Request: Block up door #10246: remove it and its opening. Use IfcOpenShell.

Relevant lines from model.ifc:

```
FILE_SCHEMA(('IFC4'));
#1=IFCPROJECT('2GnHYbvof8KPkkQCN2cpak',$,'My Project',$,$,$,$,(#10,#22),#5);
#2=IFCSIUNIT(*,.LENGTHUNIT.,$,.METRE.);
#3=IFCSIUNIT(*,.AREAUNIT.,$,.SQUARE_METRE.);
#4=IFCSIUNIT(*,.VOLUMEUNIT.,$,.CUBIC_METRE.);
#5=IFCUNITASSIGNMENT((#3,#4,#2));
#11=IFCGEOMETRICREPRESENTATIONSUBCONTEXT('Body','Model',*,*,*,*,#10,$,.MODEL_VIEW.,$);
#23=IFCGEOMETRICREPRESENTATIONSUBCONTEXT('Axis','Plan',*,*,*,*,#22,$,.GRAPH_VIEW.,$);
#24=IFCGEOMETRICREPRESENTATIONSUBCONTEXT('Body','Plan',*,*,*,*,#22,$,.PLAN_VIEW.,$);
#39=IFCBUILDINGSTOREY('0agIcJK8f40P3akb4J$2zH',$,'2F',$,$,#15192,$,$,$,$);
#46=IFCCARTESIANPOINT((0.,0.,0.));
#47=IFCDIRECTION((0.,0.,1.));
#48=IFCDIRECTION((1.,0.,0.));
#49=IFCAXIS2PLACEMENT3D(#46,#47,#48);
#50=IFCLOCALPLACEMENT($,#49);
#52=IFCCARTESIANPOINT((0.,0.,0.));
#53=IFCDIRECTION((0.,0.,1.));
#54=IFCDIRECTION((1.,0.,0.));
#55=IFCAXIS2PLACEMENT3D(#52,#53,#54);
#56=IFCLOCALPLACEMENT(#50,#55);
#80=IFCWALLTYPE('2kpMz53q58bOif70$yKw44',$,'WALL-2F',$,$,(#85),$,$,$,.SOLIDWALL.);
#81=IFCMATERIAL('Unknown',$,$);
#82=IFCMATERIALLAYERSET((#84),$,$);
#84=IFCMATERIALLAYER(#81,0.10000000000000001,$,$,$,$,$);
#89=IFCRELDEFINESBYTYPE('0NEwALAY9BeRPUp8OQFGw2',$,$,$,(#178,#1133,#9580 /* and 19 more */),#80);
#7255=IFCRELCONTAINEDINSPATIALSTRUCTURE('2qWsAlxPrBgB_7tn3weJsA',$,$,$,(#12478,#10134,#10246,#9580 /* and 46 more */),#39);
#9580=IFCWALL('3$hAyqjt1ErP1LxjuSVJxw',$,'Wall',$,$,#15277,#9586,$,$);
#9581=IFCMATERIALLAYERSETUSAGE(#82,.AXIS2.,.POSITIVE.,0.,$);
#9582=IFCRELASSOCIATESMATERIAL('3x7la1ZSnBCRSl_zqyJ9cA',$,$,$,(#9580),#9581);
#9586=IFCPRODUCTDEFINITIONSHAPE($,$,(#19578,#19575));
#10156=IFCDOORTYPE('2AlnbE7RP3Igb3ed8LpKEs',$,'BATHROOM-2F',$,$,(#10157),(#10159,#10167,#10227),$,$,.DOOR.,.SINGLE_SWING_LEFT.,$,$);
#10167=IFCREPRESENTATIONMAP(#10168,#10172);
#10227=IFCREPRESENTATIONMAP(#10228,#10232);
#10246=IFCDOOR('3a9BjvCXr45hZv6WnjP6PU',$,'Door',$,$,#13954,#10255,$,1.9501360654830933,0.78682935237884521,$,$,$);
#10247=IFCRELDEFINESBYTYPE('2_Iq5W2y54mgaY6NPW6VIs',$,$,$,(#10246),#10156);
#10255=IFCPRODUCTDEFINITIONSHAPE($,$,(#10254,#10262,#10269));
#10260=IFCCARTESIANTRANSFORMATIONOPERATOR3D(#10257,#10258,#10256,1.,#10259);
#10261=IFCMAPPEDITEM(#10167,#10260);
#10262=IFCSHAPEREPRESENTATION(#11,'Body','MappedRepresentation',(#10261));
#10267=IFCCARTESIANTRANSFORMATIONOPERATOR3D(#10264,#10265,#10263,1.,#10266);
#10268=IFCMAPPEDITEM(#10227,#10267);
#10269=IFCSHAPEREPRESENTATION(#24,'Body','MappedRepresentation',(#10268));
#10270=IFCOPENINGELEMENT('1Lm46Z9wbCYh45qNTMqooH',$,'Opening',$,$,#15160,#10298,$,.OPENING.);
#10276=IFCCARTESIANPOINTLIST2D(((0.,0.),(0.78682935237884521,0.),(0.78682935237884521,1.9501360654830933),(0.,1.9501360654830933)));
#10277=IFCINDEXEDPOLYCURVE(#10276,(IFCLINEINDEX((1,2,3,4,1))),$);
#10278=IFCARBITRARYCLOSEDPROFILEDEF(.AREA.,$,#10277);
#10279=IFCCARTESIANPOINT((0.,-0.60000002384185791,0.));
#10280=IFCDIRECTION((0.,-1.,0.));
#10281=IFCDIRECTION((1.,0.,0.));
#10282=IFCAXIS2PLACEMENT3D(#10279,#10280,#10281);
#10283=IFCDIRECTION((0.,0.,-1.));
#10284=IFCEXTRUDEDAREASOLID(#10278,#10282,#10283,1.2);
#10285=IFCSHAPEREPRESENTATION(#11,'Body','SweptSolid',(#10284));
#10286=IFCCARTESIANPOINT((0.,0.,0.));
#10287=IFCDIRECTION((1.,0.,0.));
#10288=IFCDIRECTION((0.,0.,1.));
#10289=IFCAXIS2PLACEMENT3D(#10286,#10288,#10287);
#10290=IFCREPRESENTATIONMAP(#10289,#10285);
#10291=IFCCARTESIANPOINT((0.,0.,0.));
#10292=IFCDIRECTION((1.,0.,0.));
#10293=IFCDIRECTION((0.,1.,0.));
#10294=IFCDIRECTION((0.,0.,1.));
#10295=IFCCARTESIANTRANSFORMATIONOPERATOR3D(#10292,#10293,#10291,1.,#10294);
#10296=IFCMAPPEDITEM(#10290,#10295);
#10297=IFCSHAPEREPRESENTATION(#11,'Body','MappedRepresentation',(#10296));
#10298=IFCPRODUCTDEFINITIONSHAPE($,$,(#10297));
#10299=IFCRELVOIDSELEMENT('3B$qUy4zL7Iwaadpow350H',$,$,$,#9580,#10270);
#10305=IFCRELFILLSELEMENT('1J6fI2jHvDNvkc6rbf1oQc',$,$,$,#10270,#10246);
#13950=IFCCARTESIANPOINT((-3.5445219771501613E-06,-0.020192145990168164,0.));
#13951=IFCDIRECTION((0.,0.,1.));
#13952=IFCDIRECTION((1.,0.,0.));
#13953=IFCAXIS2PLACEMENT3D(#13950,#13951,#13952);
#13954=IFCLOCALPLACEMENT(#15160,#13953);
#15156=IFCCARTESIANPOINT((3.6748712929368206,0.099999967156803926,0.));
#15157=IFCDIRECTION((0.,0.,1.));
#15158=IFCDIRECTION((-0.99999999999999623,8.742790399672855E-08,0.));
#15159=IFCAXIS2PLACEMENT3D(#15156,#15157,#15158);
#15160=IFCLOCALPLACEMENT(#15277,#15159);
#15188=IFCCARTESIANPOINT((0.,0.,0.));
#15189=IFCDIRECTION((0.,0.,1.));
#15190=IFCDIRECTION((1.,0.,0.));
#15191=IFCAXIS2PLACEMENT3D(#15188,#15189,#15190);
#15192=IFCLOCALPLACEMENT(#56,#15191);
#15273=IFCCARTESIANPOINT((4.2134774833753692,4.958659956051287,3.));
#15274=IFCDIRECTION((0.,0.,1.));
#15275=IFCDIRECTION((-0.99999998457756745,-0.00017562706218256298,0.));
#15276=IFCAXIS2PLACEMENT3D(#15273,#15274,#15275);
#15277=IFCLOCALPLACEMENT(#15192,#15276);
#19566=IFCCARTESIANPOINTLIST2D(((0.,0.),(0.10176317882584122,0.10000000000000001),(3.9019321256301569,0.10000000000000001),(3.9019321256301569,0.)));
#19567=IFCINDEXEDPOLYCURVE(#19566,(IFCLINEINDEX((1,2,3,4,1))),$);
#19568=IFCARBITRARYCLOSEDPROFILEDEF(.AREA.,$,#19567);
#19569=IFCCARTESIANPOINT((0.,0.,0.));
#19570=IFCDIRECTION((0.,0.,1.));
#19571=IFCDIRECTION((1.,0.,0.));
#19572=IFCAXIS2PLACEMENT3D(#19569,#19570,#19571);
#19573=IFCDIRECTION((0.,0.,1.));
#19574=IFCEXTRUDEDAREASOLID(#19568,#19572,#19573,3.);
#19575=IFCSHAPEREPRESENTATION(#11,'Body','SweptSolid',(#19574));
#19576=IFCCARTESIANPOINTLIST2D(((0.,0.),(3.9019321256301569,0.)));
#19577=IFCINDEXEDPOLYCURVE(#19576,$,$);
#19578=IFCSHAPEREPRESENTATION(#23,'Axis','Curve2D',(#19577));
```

```python
import ifcopenshell
import ifcopenshell.api.feature
import ifcopenshell.api.root
import ifcopenshell.geom
import ifcopenshell.util.shape

model = ifcopenshell.open("model.ifc")
settings = ifcopenshell.geom.settings()


def volume(element):
    """Net volume in cubic metres, openings subtracted."""
    shape = ifcopenshell.geom.create_shape(settings, element)
    return ifcopenshell.util.shape.get_volume(shape.geometry)


door = model.by_guid("3a9BjvCXr45hZv6WnjP6PU")
opening = door.FillsVoids[0].RelatingOpeningElement
wall = opening.VoidsElements[0].RelatingBuildingElement
before = volume(wall)

ifcopenshell.api.root.remove_product(model, product=door)
ifcopenshell.api.feature.remove_feature(model, feature=opening)

after = volume(wall)

print(f"wall volume {before:.3f} -> {after:.3f} m3")

model.write("model_updated.ifc")
```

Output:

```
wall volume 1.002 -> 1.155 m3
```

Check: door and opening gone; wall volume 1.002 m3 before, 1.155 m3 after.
